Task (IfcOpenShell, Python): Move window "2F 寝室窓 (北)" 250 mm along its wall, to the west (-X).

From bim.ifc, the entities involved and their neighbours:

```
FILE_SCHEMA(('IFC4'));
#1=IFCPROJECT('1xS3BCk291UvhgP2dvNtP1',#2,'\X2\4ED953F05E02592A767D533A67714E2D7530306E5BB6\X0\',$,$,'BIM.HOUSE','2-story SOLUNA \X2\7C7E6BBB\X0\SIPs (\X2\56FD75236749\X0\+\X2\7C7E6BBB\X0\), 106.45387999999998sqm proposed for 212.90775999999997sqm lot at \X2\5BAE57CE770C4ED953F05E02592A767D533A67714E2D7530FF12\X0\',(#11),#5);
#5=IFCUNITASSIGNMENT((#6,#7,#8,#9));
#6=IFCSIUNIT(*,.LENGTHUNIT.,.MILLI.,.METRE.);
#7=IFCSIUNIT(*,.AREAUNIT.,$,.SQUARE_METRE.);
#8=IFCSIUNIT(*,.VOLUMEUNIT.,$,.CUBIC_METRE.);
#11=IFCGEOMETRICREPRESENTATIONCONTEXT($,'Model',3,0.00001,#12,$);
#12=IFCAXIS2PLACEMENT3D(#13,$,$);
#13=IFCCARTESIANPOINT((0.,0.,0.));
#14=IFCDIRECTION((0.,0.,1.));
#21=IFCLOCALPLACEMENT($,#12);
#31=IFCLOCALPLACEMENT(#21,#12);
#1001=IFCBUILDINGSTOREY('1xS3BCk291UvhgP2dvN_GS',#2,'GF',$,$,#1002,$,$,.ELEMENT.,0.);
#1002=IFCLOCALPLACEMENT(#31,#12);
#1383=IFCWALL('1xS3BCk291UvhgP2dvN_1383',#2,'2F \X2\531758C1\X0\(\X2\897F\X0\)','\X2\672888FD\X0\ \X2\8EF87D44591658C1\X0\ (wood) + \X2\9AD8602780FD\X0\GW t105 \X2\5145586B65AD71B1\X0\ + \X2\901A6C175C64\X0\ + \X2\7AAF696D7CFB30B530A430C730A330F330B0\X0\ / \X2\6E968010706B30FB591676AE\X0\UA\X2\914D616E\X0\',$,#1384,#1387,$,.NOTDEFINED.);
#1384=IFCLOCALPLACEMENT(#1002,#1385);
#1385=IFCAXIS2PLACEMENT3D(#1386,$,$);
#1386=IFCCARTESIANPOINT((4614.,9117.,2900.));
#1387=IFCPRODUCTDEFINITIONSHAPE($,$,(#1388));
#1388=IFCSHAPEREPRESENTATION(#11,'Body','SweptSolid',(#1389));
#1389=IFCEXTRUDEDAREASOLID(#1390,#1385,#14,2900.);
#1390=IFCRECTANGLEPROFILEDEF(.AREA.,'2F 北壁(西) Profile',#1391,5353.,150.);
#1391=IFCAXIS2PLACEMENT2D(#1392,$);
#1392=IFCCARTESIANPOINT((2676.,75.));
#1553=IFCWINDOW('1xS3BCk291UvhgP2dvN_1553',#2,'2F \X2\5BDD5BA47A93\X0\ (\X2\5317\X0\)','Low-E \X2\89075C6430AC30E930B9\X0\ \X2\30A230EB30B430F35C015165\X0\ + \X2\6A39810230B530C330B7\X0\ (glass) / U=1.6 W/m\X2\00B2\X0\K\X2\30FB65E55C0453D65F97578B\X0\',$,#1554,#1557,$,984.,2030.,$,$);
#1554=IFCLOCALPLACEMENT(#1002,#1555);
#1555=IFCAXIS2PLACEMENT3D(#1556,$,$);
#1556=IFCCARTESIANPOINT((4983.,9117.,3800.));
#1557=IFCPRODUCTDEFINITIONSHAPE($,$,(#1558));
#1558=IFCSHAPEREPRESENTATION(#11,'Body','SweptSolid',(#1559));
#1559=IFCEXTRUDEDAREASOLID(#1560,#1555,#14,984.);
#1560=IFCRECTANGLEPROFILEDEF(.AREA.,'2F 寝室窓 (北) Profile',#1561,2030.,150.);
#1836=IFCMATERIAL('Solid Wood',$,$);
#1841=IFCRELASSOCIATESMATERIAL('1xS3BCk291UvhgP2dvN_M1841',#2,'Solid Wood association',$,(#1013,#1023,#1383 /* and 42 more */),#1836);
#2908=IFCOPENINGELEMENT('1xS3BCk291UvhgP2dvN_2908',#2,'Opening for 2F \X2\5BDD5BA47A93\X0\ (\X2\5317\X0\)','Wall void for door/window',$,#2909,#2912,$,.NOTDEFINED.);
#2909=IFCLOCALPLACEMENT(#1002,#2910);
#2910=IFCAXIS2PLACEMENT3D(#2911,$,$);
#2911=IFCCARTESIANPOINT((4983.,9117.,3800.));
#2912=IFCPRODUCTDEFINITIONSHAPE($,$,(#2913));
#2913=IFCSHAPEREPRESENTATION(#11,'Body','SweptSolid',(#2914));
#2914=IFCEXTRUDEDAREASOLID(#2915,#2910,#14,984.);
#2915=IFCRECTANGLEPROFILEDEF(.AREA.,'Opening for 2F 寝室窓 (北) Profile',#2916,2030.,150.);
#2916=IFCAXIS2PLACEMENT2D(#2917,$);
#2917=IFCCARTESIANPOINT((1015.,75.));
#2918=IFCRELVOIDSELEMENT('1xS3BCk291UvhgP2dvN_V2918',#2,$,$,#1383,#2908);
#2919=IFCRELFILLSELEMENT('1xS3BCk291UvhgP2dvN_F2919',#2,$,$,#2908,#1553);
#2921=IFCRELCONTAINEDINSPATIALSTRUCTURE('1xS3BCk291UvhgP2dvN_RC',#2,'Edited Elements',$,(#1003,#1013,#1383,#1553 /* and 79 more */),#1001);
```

```python
import ifcopenshell
import ifcopenshell.api.geometry
import ifcopenshell.util.placement
import ifcopenshell.util.unit

model = ifcopenshell.open("bim.ifc")
unit_scale = ifcopenshell.util.unit.calculate_unit_scale(model)

window = model.by_guid("1xS3BCk291UvhgP2dvN_1553")
opening = window.FillsVoids[0].RelatingOpeningElement
wall = opening.VoidsElements[0].RelatingBuildingElement

wall_matrix = ifcopenshell.util.placement.get_local_placement(wall.ObjectPlacement)
shift = wall_matrix[:3, 0] * -0.25 / unit_scale
before = ifcopenshell.util.placement.get_local_placement(window.ObjectPlacement)[:3, 3].copy()

# The window is not placed relative to its opening, so move both.
for product in (opening, window):
    matrix = ifcopenshell.util.placement.get_local_placement(product.ObjectPlacement)
    matrix[:3, 3] += shift
    ifcopenshell.api.geometry.edit_object_placement(model, product=product, matrix=matrix, is_si=False)

after = ifcopenshell.util.placement.get_local_placement(window.ObjectPlacement)[:3, 3]
print("window moved by", (after - before).round(3) + 0.0)

model.write("bim_updated.ifc")
```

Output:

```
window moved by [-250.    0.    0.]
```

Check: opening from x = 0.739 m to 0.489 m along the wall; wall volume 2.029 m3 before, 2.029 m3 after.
